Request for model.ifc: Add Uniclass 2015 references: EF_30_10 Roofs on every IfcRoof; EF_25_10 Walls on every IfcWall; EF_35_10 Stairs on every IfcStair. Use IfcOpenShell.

First a look at what the model holds.

```python
import ifcopenshell

model = ifcopenshell.open("model.ifc")
print(model.schema)
print("classifications:", [c.Name for c in model.by_type("IfcClassification")])
for ifc_class in ("IfcDoor", "IfcRoof", "IfcStair", "IfcWall", "IfcWindow"):
    print(ifc_class, len(model.by_type(ifc_class)))
```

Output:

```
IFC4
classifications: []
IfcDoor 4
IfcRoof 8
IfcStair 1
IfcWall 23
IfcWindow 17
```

```python
import ifcopenshell
import ifcopenshell.api.classification

model = ifcopenshell.open("model.ifc")

system = ifcopenshell.api.classification.add_classification(model, classification="Uniclass 2015")

codes = {
    "IfcRoof": ("EF_30_10", "Roofs"),
    "IfcWall": ("EF_25_10", "Walls"),
    "IfcStair": ("EF_35_10", "Stairs"),
}
for ifc_class, (code, name) in codes.items():
    products = model.by_type(ifc_class)
    ifcopenshell.api.classification.add_reference(
        model, products=products, classification=system, identification=code, name=name
    )
    print(code, len(products))

model.write("model_rev.ifc")
```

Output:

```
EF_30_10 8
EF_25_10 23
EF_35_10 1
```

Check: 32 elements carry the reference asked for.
